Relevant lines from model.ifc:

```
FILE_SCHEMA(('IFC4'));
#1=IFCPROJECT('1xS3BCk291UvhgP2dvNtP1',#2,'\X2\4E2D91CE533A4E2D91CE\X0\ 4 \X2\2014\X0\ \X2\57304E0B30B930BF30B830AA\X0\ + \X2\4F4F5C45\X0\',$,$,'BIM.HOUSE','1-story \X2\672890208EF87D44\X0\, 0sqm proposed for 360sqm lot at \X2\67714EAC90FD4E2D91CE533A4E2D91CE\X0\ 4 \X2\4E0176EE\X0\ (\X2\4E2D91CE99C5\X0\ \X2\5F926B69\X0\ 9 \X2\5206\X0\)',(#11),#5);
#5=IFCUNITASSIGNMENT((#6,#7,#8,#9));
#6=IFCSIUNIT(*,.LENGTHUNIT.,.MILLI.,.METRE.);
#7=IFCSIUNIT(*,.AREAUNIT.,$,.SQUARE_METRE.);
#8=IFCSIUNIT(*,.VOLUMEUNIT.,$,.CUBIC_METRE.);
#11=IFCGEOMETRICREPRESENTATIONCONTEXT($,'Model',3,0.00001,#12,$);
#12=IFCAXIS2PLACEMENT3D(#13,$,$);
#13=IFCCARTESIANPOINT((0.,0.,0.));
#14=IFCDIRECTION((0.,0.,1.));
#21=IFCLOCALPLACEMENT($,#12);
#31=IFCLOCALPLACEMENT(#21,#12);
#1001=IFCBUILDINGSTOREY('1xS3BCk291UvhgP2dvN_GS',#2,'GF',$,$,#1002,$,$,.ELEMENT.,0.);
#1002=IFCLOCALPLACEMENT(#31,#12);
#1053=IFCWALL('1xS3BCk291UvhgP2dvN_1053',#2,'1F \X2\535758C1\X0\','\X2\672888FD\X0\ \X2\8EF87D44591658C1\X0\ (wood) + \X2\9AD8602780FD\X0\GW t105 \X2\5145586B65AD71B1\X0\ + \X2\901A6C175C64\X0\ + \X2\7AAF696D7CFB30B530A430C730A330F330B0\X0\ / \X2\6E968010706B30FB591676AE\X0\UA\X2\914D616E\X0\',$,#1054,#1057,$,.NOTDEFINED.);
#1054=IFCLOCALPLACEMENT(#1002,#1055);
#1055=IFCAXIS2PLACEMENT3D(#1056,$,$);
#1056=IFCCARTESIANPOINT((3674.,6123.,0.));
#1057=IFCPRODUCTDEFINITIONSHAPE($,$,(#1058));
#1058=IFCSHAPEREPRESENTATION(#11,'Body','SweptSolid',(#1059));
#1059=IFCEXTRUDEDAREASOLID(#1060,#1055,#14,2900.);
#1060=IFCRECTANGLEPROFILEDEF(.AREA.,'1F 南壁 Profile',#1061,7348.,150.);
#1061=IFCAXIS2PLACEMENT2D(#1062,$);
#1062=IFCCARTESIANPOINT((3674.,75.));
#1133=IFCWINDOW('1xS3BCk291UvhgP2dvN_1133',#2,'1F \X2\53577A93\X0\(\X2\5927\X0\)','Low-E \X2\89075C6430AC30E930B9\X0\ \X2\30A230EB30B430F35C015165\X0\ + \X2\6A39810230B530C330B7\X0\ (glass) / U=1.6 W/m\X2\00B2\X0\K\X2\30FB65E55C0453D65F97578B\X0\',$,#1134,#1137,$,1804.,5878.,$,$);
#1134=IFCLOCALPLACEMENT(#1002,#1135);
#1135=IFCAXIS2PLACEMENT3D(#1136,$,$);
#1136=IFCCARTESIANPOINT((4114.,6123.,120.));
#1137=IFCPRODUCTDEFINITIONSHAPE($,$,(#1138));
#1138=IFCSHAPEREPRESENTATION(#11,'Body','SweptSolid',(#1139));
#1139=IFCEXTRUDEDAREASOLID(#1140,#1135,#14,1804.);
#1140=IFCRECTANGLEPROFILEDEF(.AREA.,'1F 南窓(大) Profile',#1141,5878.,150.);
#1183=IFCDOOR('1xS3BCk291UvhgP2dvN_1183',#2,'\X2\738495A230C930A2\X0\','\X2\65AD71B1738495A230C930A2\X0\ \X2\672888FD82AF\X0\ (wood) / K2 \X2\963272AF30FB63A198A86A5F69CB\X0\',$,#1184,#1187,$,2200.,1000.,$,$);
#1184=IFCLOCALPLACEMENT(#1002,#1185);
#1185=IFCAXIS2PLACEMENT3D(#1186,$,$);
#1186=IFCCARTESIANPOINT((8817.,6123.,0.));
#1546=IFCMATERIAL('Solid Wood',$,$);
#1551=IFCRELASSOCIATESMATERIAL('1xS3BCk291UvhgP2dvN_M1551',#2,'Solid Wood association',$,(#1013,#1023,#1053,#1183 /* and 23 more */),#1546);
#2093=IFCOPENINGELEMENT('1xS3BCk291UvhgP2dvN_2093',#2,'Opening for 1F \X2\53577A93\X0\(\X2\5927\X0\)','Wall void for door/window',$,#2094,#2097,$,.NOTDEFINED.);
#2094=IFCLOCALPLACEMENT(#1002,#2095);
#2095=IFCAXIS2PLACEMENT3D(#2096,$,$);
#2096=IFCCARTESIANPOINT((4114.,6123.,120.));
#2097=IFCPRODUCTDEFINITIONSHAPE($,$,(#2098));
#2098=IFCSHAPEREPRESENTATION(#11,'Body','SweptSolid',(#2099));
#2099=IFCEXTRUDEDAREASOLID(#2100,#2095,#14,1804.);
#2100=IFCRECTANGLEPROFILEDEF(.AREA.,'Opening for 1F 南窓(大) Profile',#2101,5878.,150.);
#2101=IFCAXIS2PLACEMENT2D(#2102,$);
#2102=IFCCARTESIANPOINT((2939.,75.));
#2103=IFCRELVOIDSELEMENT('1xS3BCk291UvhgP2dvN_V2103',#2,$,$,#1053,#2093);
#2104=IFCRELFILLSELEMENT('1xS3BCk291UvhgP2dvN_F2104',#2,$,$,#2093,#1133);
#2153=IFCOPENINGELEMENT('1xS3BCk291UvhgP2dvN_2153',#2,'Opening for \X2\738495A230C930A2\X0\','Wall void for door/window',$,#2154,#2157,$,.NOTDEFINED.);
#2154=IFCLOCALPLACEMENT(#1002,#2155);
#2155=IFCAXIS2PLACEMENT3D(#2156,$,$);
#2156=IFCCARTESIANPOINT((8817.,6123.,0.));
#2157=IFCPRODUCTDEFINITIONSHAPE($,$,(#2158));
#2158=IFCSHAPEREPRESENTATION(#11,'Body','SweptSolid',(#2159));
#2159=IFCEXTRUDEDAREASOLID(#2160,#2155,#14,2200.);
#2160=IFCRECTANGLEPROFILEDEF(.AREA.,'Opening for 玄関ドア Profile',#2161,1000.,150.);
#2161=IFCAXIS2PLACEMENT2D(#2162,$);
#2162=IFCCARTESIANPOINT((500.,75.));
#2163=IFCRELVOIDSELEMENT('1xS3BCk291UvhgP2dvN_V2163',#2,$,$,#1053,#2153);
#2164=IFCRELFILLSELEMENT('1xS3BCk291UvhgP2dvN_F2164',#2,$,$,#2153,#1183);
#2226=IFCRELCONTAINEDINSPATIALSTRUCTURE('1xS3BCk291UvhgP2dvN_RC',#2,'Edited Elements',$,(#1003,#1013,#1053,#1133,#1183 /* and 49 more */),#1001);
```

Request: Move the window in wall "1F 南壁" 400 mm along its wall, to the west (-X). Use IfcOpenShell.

```python
import ifcopenshell
import ifcopenshell.api.geometry
import ifcopenshell.util.placement
import ifcopenshell.util.unit

model = ifcopenshell.open("model.ifc")
unit_scale = ifcopenshell.util.unit.calculate_unit_scale(model)

window = model.by_guid("1xS3BCk291UvhgP2dvN_1133")
opening = window.FillsVoids[0].RelatingOpeningElement
wall = opening.VoidsElements[0].RelatingBuildingElement

wall_matrix = ifcopenshell.util.placement.get_local_placement(wall.ObjectPlacement)
shift = wall_matrix[:3, 0] * -0.4 / unit_scale
before = ifcopenshell.util.placement.get_local_placement(window.ObjectPlacement)[:3, 3].copy()

# The window is not placed relative to its opening, so move both.
for product in (opening, window):
    matrix = ifcopenshell.util.placement.get_local_placement(product.ObjectPlacement)
    matrix[:3, 3] += shift
    ifcopenshell.api.geometry.edit_object_placement(model, product=product, matrix=matrix, is_si=False)

after = ifcopenshell.util.placement.get_local_placement(window.ObjectPlacement)[:3, 3]
print("window moved by", (after - before).round(3) + 0.0)

model.write("model_updated.ifc")
```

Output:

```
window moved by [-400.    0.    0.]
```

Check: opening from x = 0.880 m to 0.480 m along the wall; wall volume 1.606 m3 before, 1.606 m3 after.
